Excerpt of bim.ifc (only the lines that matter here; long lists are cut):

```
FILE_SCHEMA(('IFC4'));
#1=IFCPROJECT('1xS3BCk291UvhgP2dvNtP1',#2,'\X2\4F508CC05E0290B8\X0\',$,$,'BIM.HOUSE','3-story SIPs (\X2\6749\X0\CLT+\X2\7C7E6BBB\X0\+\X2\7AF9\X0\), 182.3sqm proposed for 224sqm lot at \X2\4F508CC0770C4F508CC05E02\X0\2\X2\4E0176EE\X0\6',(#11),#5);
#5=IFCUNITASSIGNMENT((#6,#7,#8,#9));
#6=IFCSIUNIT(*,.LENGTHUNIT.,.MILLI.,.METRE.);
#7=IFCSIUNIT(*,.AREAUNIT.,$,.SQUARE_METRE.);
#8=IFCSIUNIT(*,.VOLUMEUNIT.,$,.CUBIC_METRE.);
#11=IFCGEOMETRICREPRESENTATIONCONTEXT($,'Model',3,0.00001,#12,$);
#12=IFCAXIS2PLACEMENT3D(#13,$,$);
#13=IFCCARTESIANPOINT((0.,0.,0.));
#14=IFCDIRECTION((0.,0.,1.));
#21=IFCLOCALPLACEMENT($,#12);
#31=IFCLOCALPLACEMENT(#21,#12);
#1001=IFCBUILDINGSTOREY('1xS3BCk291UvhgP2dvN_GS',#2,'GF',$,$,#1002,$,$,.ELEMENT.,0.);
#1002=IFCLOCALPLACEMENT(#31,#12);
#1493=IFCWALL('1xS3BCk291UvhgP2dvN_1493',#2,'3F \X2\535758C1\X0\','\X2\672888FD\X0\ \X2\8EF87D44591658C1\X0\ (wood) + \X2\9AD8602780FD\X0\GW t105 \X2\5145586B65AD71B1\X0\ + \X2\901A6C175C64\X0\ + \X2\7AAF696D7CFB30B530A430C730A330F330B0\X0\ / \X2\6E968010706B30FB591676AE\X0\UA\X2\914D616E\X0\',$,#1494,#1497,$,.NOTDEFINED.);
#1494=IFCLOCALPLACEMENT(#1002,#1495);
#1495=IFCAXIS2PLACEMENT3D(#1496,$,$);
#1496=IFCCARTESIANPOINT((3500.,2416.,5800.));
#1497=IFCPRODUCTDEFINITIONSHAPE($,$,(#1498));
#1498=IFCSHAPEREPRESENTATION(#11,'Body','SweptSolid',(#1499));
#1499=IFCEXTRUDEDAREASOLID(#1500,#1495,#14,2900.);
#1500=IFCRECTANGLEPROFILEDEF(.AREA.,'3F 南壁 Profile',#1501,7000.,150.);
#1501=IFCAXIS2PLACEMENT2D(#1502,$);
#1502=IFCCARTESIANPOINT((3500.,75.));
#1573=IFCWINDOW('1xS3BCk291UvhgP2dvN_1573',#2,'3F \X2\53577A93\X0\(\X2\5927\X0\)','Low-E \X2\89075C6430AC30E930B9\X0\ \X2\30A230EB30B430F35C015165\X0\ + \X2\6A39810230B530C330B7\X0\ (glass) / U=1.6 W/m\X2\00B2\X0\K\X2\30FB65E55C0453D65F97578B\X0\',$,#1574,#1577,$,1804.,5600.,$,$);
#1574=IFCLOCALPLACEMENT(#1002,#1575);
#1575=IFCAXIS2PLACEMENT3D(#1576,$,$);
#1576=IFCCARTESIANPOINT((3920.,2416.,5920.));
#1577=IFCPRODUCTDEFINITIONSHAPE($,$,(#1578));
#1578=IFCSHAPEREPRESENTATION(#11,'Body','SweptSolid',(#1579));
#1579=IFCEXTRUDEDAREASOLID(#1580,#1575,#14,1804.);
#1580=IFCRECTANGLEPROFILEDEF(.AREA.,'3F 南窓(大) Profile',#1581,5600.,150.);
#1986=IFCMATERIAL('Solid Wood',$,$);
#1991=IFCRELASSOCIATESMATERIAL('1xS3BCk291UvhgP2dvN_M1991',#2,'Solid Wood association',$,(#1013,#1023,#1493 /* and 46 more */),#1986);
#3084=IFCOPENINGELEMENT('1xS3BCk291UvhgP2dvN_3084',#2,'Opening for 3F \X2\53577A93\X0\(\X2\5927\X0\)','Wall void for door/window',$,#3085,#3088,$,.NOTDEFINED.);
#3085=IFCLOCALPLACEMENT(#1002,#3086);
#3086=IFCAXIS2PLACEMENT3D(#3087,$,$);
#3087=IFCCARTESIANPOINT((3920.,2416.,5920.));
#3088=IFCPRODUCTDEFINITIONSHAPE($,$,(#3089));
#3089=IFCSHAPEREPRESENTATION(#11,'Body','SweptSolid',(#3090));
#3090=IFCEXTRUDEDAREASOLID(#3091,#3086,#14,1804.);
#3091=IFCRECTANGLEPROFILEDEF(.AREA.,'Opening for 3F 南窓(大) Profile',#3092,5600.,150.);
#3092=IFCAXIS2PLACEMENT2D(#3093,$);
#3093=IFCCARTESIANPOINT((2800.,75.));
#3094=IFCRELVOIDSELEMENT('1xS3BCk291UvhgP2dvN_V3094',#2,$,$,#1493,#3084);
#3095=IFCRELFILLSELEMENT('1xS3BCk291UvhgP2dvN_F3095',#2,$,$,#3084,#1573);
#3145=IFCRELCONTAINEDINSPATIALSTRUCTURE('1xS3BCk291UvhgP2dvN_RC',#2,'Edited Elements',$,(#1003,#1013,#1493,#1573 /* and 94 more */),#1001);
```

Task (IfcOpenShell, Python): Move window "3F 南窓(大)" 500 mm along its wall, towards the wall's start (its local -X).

```python
import ifcopenshell
import ifcopenshell.api.geometry
import ifcopenshell.util.placement
import ifcopenshell.util.unit

model = ifcopenshell.open("bim.ifc")
unit_scale = ifcopenshell.util.unit.calculate_unit_scale(model)

window = model.by_id(1573)
opening = window.FillsVoids[0].RelatingOpeningElement
wall = opening.VoidsElements[0].RelatingBuildingElement

wall_matrix = ifcopenshell.util.placement.get_local_placement(wall.ObjectPlacement)
shift = wall_matrix[:3, 0] * -0.5 / unit_scale
before = ifcopenshell.util.placement.get_local_placement(window.ObjectPlacement)[:3, 3].copy()

# The window is not placed relative to its opening, so move both.
for product in (opening, window):
    matrix = ifcopenshell.util.placement.get_local_placement(product.ObjectPlacement)
    matrix[:3, 3] += shift
    ifcopenshell.api.geometry.edit_object_placement(model, product=product, matrix=matrix, is_si=False)

after = ifcopenshell.util.placement.get_local_placement(window.ObjectPlacement)[:3, 3]
print("window moved by", (after - before).round(3) + 0.0)

model.write("bim-out.ifc")
```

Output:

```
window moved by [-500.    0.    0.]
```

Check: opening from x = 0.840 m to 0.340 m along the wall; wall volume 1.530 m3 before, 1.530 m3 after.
